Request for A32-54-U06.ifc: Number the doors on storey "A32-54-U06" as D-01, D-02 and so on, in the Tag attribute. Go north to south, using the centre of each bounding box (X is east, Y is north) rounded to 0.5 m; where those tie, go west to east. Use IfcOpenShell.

First a look at what the model holds.

```python
import ifcopenshell
import ifcopenshell.util.element
import ifcopenshell.util.placement

model = ifcopenshell.open("A32-54-U06.ifc")
print(model.schema)
storey = next(s for s in model.by_type("IfcBuildingStorey") if s.Name == "A32-54-U06")
doors = [e for e in ifcopenshell.util.element.get_decomposition(storey) if e.is_a("IfcDoor")]
for e in sorted(doors, key=lambda e: e.id()):
    origin = ifcopenshell.util.placement.get_local_placement(e.ObjectPlacement)[:3, 3]
    print(e.id(), e.Tag, e.Name, origin.round(2) + 0.0, sep=" | ")
```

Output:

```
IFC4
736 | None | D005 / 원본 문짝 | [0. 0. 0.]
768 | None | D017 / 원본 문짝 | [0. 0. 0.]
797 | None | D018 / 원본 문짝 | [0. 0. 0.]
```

```python
import ifcopenshell
import ifcopenshell.geom
import ifcopenshell.util.element
import ifcopenshell.util.shape

model = ifcopenshell.open("A32-54-U06.ifc")
settings = ifcopenshell.geom.settings()
settings.set("use-world-coords", True)


def centre(element):
    shape = ifcopenshell.geom.create_shape(settings, element)
    return ifcopenshell.util.shape.get_bbox_centroid(shape.geometry)


storey = next(s for s in model.by_type("IfcBuildingStorey") if s.Name == "A32-54-U06")
doors = [e for e in ifcopenshell.util.element.get_decomposition(storey) if e.is_a("IfcDoor")]

# Insertion points can sit at a corner or the storey origin, so sort by the geometry (in metres).
centres = {e: centre(e) for e in doors}
doors.sort(key=lambda e: (-round(centres[e][1] / 0.5), centres[e][0]))

for i, e in enumerate(doors, start=1):
    number = f"D-{i:02d}"
    e.Tag = number
    print(e.id(), number)

model.write("A32-54-U06_edited.ifc")
```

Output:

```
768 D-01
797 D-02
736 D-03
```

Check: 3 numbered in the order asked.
